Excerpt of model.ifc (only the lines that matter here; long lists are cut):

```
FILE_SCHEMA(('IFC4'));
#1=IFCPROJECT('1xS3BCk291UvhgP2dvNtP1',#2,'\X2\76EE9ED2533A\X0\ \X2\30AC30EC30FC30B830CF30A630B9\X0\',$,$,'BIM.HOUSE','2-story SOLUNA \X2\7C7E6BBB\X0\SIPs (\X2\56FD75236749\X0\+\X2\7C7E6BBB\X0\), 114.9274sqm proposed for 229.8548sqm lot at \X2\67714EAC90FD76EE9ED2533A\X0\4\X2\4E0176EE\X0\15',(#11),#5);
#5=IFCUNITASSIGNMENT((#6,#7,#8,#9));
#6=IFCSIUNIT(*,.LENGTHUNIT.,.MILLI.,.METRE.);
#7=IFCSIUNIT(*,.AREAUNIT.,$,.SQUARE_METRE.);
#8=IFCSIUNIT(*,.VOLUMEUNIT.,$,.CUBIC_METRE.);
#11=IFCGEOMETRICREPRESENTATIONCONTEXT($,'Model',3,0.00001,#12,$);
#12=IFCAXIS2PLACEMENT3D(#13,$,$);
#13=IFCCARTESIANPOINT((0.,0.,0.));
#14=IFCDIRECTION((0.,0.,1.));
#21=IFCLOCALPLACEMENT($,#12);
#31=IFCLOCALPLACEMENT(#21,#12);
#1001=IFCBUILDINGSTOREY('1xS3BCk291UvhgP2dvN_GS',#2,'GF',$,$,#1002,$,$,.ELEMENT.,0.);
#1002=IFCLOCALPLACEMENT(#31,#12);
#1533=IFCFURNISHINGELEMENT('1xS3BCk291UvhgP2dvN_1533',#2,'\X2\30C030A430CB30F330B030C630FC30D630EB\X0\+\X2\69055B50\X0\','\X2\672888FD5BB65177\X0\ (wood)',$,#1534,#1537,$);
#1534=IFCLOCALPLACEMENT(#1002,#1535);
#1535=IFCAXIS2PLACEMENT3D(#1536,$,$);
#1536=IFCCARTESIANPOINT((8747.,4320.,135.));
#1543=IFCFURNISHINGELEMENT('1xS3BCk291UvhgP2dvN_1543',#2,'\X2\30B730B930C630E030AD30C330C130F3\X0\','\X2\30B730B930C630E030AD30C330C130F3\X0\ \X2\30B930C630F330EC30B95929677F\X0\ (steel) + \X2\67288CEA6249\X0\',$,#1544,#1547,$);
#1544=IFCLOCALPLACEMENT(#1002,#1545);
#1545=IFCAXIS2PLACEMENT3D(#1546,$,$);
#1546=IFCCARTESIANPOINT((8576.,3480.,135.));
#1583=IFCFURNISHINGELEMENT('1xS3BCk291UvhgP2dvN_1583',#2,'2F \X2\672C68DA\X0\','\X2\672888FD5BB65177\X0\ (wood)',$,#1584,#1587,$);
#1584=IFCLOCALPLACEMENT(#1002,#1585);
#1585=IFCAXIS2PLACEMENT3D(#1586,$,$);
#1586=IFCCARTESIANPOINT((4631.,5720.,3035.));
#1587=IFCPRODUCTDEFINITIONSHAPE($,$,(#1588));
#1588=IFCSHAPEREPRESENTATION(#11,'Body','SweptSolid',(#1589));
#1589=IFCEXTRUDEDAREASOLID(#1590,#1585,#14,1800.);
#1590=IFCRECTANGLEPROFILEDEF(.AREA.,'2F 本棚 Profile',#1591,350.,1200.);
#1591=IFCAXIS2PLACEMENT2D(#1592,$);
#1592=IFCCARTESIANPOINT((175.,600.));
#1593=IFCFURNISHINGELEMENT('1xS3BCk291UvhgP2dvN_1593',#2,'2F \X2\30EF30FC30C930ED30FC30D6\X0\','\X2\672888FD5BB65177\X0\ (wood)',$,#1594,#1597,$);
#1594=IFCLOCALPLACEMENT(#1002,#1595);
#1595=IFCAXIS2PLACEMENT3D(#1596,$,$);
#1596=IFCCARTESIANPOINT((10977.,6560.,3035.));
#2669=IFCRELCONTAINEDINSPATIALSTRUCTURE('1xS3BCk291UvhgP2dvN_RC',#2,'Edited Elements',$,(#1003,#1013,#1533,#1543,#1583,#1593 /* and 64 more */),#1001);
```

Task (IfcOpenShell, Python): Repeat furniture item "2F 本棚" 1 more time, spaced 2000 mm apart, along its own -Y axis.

```python
import ifcopenshell
import ifcopenshell.api.geometry
import ifcopenshell.api.root
import ifcopenshell.util.element
import ifcopenshell.util.placement
import ifcopenshell.util.unit

model = ifcopenshell.open("model.ifc")
unit_scale = ifcopenshell.util.unit.calculate_unit_scale(model)


def reuse_history(source, copy):
    """copy_class also copies each property set's owner history, people and application; keep the originals."""
    for rel in copy.IsDefinedBy:
        if rel.is_a("IfcRelDefinesByProperties") and (history := rel.RelatingPropertyDefinition.OwnerHistory):
            rel.RelatingPropertyDefinition.OwnerHistory = source.OwnerHistory
            ifcopenshell.util.element.remove_deep2(model, history)


source = model.by_guid("1xS3BCk291UvhgP2dvN_1583")
base = ifcopenshell.util.placement.get_local_placement(source.ObjectPlacement)
step = -base[:3, 1] * 2 / unit_scale

for i in range(1, 2):
    copy = ifcopenshell.api.root.copy_class(model, product=source)
    copy.Representation = ifcopenshell.util.element.copy_deep(
        model, source.Representation, exclude=["IfcGeometricRepresentationContext", "IfcRepresentationMap"]
    )
    reuse_history(source, copy)
    matrix = base.copy()
    matrix[:3, 3] += i * step
    print("added at", matrix[:3, 3].round(3) + 0.0)
    ifcopenshell.api.geometry.edit_object_placement(model, product=copy, matrix=matrix, is_si=False)

model.write("model_rev.ifc")
```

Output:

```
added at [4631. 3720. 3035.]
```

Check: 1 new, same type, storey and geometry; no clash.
